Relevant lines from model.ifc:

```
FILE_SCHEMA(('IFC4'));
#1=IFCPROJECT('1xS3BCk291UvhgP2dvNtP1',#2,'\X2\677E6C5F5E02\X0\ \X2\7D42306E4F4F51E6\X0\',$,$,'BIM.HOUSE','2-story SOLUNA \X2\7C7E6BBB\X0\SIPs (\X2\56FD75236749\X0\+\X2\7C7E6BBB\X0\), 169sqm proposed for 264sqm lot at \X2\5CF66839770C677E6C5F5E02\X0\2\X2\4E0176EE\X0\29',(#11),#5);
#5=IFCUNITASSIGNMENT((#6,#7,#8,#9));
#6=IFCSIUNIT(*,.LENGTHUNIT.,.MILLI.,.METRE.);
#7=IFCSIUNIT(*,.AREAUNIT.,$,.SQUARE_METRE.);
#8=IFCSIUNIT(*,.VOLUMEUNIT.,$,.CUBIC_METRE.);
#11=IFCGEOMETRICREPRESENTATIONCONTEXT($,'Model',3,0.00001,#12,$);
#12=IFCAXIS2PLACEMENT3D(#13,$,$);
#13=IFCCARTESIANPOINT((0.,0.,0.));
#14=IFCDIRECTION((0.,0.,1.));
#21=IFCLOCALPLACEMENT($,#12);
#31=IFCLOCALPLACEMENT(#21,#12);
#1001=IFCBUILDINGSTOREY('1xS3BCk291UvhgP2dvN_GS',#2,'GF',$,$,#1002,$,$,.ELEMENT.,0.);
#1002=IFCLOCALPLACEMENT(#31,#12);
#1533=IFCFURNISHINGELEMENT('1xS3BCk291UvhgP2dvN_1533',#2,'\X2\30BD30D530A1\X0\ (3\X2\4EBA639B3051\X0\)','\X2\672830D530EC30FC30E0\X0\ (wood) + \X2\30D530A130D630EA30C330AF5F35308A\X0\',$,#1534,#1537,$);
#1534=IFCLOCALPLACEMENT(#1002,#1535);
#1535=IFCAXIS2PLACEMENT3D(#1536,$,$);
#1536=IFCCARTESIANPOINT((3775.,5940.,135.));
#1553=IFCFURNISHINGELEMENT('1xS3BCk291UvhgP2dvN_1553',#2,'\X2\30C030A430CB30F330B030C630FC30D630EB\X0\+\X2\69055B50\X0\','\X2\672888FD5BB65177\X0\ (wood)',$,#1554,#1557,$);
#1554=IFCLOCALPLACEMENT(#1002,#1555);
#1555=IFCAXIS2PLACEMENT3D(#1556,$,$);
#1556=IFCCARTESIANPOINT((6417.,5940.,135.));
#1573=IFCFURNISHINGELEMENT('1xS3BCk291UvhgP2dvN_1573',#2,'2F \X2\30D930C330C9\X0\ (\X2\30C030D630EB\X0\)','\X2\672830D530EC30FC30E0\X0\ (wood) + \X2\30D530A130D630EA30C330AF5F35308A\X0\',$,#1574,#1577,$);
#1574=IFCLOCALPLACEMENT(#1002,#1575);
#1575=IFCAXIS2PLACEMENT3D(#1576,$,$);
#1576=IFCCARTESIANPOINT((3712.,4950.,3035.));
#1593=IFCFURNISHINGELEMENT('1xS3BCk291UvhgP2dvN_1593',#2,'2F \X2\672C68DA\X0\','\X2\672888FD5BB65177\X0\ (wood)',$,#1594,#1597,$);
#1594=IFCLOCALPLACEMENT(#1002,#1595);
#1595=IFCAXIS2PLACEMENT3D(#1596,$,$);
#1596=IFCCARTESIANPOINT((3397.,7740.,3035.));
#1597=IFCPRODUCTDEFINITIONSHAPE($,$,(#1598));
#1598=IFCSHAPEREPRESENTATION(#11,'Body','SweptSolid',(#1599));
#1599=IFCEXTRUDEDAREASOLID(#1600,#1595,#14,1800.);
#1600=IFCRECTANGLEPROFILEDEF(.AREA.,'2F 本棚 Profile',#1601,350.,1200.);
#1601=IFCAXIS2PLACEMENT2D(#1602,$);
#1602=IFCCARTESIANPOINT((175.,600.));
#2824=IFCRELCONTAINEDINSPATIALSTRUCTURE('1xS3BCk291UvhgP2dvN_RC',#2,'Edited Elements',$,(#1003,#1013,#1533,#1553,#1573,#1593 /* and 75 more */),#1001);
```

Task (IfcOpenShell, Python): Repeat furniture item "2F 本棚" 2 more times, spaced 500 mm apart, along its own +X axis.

```python
import ifcopenshell
import ifcopenshell.api.geometry
import ifcopenshell.api.root
import ifcopenshell.util.element
import ifcopenshell.util.placement
import ifcopenshell.util.unit

model = ifcopenshell.open("model.ifc")
unit_scale = ifcopenshell.util.unit.calculate_unit_scale(model)


def reuse_history(source, copy):
    """copy_class also copies each property set's owner history, people and application; keep the originals."""
    for rel in copy.IsDefinedBy:
        if rel.is_a("IfcRelDefinesByProperties") and (history := rel.RelatingPropertyDefinition.OwnerHistory):
            rel.RelatingPropertyDefinition.OwnerHistory = source.OwnerHistory
            ifcopenshell.util.element.remove_deep2(model, history)


source = model.by_guid("1xS3BCk291UvhgP2dvN_1593")
base = ifcopenshell.util.placement.get_local_placement(source.ObjectPlacement)
step = base[:3, 0] * 0.5 / unit_scale

for i in range(1, 3):
    copy = ifcopenshell.api.root.copy_class(model, product=source)
    copy.Representation = ifcopenshell.util.element.copy_deep(
        model, source.Representation, exclude=["IfcGeometricRepresentationContext", "IfcRepresentationMap"]
    )
    reuse_history(source, copy)
    matrix = base.copy()
    matrix[:3, 3] += i * step
    print("added at", matrix[:3, 3].round(3) + 0.0)
    ifcopenshell.api.geometry.edit_object_placement(model, product=copy, matrix=matrix, is_si=False)

model.write("model_edited.ifc")
```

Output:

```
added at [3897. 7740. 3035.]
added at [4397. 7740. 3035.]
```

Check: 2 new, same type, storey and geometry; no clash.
